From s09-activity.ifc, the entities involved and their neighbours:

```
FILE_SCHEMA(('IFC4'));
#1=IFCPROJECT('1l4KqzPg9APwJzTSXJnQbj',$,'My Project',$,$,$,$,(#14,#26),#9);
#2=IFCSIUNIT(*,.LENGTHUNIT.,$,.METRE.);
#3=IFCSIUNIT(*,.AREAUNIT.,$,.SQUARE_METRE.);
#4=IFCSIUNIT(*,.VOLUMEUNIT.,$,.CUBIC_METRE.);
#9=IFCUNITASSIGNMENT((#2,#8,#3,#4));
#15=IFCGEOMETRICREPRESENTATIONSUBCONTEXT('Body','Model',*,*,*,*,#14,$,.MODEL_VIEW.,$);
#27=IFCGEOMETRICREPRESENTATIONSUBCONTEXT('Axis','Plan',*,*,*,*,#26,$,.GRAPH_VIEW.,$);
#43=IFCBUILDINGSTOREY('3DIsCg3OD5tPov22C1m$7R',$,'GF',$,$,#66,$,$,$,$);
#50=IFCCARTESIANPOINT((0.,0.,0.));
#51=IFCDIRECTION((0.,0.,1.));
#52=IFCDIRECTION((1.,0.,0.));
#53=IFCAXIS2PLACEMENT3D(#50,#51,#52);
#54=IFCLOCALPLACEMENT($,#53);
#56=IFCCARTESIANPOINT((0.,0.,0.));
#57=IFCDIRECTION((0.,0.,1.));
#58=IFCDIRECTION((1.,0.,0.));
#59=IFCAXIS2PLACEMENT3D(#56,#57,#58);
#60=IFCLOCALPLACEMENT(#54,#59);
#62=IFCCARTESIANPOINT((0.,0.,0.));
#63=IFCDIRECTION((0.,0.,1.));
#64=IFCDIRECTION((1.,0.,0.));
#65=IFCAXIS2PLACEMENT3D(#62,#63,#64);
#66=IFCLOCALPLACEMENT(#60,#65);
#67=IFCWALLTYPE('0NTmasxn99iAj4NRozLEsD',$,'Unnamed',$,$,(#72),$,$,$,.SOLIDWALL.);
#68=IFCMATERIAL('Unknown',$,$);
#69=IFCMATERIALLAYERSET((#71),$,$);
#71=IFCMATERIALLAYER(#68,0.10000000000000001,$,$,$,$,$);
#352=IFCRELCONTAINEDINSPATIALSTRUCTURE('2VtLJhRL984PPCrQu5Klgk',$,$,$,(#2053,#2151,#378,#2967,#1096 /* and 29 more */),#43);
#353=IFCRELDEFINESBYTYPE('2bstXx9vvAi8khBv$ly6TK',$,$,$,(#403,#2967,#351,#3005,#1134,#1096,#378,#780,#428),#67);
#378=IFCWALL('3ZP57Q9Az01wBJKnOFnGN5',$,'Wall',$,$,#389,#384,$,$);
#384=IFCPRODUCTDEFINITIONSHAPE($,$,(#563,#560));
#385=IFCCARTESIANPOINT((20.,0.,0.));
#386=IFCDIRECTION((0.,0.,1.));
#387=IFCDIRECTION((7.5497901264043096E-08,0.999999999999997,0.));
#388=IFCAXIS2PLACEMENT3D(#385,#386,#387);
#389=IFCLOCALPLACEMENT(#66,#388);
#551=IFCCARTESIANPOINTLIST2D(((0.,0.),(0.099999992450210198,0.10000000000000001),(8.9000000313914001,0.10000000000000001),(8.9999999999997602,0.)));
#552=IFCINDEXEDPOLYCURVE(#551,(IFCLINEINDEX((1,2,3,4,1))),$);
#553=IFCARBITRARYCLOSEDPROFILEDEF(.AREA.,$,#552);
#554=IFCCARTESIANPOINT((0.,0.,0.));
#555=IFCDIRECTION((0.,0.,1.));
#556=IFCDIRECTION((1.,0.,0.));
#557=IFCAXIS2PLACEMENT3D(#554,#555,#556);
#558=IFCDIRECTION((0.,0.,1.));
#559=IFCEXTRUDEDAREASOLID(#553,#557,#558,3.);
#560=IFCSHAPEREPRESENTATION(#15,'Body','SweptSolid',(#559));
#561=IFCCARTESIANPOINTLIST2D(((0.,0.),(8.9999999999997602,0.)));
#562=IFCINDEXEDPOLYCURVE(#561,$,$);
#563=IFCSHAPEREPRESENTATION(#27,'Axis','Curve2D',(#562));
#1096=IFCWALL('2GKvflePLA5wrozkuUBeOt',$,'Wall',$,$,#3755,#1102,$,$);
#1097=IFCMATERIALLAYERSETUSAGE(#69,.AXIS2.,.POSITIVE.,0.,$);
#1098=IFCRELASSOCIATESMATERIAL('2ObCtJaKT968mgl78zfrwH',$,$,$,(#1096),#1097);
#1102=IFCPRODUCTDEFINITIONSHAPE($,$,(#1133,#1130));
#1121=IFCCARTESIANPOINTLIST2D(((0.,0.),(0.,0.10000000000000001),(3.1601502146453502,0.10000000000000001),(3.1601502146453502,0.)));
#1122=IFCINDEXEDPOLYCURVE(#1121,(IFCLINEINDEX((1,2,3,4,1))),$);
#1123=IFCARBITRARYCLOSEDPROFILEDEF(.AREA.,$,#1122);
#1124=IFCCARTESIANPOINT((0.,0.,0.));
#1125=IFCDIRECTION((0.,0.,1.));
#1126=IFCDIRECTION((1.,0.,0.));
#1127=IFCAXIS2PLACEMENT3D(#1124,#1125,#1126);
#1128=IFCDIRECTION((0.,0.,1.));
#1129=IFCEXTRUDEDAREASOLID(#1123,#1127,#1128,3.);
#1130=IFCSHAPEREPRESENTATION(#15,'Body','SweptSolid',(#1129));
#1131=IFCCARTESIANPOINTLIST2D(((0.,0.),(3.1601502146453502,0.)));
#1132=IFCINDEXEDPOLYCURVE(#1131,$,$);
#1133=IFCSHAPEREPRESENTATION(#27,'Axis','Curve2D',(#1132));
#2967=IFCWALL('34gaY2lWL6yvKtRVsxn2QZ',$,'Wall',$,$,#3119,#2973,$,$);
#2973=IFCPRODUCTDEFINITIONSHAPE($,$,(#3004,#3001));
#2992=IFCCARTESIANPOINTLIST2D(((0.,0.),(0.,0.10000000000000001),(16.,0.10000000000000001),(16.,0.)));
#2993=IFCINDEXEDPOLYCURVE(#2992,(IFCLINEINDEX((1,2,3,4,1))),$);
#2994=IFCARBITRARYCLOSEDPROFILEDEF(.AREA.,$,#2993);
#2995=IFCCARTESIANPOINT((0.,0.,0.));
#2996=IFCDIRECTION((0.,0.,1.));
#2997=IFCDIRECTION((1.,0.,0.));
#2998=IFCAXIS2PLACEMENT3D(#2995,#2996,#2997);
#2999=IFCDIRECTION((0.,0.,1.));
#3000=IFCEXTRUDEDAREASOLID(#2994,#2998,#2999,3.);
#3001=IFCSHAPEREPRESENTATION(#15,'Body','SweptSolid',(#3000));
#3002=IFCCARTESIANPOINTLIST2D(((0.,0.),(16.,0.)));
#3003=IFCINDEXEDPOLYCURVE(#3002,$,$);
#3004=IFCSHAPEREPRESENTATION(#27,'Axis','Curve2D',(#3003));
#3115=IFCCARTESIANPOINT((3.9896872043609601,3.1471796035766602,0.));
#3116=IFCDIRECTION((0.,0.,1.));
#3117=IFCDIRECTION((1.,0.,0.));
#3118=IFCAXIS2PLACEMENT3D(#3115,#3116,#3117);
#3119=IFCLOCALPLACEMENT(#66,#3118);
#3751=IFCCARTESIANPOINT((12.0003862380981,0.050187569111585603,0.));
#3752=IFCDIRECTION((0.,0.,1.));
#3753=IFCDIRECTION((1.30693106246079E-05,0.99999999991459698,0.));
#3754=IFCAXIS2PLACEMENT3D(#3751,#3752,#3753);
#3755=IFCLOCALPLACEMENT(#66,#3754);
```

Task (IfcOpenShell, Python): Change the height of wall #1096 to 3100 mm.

```python
import ifcopenshell
import ifcopenshell.geom
import ifcopenshell.util.representation
import ifcopenshell.util.shape
import ifcopenshell.util.unit

model = ifcopenshell.open("s09-activity.ifc")
unit_scale = ifcopenshell.util.unit.calculate_unit_scale(model)
settings = ifcopenshell.geom.settings()


def volume(element):
    """Net volume in cubic metres, openings subtracted."""
    shape = ifcopenshell.geom.create_shape(settings, element)
    return ifcopenshell.util.shape.get_volume(shape.geometry)


wall = model.by_guid("2GKvflePLA5wrozkuUBeOt")
before = volume(wall)

body = ifcopenshell.util.representation.get_representation(wall, "Model", "Body")
solid = body.Items[0]
old_height = solid.Depth
solid.Depth = 3.1 / unit_scale
after = volume(wall)

print(f"height {old_height:g} -> {solid.Depth:g}, volume {before:.3f} -> {after:.3f} m3")

model.write("s09-activity_edited.ifc")
```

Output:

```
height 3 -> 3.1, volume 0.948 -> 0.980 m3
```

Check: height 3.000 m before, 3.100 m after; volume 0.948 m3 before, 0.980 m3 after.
